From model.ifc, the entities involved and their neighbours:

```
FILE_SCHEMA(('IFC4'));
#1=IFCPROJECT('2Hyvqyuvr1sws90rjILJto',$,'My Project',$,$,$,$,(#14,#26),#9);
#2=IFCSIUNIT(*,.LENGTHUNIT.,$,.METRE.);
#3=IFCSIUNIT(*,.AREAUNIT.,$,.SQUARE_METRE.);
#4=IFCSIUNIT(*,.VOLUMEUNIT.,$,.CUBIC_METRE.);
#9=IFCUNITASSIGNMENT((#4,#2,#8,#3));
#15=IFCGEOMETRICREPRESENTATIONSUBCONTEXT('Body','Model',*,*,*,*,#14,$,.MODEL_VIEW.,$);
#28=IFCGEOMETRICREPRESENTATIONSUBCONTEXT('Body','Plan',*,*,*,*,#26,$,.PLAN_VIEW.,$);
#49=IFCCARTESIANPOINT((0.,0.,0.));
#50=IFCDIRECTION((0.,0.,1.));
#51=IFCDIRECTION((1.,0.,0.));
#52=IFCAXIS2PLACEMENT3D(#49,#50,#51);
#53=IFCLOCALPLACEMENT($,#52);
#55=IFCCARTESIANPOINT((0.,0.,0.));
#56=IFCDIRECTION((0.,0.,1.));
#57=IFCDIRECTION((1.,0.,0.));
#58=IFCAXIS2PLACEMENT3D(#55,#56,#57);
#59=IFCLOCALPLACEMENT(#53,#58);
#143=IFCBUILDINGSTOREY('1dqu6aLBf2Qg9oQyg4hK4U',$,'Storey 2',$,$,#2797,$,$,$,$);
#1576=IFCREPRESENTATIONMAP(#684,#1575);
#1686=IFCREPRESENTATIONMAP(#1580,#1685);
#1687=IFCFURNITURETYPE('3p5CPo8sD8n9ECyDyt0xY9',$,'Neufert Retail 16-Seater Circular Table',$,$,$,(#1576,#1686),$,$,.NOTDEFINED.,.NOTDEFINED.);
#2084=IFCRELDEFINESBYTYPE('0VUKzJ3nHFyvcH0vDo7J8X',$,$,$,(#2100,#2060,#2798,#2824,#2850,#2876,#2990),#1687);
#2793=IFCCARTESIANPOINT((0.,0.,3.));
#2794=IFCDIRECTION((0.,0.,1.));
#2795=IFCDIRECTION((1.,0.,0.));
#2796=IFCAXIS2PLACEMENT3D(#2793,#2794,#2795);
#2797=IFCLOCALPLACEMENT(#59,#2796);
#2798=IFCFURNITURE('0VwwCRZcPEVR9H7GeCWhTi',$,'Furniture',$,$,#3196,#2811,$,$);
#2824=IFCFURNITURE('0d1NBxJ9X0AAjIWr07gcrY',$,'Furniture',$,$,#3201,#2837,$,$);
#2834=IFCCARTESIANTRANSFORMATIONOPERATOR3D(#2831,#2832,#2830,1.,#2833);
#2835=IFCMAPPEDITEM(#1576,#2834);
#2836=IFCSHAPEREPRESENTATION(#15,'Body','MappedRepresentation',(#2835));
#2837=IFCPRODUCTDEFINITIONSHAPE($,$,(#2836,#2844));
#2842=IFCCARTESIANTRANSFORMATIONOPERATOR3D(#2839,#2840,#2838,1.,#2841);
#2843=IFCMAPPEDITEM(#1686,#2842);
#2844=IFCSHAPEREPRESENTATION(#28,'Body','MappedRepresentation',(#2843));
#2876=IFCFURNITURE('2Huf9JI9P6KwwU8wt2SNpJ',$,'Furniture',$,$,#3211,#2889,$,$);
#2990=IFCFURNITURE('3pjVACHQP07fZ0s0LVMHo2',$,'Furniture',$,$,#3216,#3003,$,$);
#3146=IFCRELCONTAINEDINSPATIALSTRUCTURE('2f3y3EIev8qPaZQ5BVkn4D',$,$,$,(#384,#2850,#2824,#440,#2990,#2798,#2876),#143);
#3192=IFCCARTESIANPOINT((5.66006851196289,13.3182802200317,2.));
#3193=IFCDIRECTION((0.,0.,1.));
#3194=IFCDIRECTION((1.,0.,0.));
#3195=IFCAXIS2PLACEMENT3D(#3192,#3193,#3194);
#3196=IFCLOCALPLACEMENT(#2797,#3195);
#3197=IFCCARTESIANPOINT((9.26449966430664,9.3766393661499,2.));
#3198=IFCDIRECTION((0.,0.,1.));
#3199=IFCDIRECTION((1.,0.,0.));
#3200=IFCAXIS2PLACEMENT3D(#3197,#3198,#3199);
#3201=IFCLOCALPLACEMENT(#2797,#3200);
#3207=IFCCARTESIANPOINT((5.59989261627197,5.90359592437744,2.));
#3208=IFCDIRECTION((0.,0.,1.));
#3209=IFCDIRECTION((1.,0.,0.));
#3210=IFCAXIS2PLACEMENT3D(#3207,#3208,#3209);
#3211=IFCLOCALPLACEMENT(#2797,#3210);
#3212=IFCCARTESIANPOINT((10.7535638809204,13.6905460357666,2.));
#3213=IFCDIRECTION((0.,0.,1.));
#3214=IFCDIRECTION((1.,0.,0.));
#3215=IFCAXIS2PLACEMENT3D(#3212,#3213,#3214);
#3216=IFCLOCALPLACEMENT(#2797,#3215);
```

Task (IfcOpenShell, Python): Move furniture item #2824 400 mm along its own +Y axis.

```python
import ifcopenshell
import ifcopenshell.api.geometry
import ifcopenshell.util.placement

model = ifcopenshell.open("model.ifc")

item = model.by_guid("0d1NBxJ9X0AAjIWr07gcrY")
matrix = ifcopenshell.util.placement.get_local_placement(item.ObjectPlacement)
matrix[:3, 3] += matrix[:3, 1] * 0.4
ifcopenshell.api.geometry.edit_object_placement(model, product=item, matrix=matrix, is_si=False)

print(ifcopenshell.util.placement.get_local_placement(item.ObjectPlacement).round(3) + 0.0)

model.write("model_v2.ifc")
```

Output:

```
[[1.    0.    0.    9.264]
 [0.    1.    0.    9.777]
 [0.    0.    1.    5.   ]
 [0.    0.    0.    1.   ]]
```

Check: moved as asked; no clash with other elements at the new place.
